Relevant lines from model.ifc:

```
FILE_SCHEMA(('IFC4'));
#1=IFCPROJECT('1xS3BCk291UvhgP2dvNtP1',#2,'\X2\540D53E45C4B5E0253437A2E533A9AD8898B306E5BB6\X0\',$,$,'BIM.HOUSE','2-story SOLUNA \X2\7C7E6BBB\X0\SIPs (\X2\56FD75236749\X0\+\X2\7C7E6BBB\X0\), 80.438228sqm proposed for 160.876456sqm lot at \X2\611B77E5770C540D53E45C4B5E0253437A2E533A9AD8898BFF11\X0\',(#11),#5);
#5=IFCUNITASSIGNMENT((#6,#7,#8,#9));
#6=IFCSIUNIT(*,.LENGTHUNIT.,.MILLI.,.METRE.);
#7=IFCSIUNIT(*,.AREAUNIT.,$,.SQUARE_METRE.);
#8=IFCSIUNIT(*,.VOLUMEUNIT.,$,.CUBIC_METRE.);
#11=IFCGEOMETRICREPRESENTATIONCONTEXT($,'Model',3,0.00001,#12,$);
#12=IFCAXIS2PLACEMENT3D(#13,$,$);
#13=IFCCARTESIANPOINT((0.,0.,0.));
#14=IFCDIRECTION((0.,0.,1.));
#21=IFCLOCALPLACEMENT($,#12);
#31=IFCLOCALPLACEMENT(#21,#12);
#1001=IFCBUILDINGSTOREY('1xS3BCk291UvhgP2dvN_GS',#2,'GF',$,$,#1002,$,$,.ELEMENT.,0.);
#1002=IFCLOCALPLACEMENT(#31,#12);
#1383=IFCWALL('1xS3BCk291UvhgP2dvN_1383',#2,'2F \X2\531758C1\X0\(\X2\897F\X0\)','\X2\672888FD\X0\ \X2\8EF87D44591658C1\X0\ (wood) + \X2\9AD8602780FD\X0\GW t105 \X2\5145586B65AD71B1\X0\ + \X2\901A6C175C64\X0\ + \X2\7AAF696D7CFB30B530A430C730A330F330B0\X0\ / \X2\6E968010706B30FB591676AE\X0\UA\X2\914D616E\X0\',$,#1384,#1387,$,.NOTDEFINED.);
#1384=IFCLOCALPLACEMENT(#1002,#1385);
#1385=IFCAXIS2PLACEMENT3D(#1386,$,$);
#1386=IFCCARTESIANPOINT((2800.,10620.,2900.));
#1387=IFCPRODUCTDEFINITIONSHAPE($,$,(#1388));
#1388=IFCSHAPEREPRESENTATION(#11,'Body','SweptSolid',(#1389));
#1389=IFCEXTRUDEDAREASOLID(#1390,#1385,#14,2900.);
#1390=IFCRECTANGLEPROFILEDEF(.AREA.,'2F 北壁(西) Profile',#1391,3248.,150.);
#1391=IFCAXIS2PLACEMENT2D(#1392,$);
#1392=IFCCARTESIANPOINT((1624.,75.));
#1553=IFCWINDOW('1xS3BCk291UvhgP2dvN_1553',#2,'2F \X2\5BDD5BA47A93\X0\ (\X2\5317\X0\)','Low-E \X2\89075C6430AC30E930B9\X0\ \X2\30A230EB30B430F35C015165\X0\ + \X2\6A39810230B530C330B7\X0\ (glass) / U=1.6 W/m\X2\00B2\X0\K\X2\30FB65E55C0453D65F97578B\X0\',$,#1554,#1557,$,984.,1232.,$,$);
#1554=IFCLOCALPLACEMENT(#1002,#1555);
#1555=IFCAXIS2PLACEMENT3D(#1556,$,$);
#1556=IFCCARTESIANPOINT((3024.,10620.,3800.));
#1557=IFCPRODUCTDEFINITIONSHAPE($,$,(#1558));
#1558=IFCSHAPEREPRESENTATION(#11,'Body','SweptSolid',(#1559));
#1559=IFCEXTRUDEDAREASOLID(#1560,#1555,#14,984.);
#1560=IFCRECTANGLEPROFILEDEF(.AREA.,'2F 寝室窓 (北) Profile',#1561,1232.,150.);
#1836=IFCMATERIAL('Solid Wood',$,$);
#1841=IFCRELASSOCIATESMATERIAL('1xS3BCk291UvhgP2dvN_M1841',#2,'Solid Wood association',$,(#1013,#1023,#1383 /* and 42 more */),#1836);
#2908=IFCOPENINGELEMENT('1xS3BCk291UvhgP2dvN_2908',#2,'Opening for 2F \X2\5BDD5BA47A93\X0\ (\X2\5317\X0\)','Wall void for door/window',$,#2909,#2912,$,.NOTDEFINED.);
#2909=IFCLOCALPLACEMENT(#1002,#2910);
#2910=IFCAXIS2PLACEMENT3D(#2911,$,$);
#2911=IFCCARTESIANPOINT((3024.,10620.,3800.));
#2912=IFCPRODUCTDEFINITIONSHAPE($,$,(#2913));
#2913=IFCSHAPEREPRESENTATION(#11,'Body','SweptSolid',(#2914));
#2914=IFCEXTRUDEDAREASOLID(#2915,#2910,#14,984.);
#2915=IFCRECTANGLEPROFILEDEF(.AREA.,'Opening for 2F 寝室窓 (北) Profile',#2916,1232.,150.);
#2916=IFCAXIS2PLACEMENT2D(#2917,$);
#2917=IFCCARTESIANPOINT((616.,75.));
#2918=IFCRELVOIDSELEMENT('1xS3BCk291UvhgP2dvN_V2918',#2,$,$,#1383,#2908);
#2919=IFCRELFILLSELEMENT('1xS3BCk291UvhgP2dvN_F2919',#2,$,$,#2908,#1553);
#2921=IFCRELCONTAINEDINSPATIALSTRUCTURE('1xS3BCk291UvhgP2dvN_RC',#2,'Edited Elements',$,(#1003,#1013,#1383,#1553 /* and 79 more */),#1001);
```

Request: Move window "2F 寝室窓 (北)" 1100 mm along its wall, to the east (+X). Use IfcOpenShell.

```python
import ifcopenshell
import ifcopenshell.api.geometry
import ifcopenshell.util.placement
import ifcopenshell.util.unit

model = ifcopenshell.open("model.ifc")
unit_scale = ifcopenshell.util.unit.calculate_unit_scale(model)

window = model.by_id(1553)
opening = window.FillsVoids[0].RelatingOpeningElement
wall = opening.VoidsElements[0].RelatingBuildingElement

wall_matrix = ifcopenshell.util.placement.get_local_placement(wall.ObjectPlacement)
shift = wall_matrix[:3, 0] * 1.1 / unit_scale
before = ifcopenshell.util.placement.get_local_placement(window.ObjectPlacement)[:3, 3].copy()

# The window is not placed relative to its opening, so move both.
for product in (opening, window):
    matrix = ifcopenshell.util.placement.get_local_placement(product.ObjectPlacement)
    matrix[:3, 3] += shift
    ifcopenshell.api.geometry.edit_object_placement(model, product=product, matrix=matrix, is_si=False)

after = ifcopenshell.util.placement.get_local_placement(window.ObjectPlacement)[:3, 3]
print("window moved by", (after - before).round(3) + 0.0)

model.write("model-out.ifc")
```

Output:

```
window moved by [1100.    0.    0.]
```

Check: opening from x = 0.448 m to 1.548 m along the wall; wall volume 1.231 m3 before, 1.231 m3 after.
